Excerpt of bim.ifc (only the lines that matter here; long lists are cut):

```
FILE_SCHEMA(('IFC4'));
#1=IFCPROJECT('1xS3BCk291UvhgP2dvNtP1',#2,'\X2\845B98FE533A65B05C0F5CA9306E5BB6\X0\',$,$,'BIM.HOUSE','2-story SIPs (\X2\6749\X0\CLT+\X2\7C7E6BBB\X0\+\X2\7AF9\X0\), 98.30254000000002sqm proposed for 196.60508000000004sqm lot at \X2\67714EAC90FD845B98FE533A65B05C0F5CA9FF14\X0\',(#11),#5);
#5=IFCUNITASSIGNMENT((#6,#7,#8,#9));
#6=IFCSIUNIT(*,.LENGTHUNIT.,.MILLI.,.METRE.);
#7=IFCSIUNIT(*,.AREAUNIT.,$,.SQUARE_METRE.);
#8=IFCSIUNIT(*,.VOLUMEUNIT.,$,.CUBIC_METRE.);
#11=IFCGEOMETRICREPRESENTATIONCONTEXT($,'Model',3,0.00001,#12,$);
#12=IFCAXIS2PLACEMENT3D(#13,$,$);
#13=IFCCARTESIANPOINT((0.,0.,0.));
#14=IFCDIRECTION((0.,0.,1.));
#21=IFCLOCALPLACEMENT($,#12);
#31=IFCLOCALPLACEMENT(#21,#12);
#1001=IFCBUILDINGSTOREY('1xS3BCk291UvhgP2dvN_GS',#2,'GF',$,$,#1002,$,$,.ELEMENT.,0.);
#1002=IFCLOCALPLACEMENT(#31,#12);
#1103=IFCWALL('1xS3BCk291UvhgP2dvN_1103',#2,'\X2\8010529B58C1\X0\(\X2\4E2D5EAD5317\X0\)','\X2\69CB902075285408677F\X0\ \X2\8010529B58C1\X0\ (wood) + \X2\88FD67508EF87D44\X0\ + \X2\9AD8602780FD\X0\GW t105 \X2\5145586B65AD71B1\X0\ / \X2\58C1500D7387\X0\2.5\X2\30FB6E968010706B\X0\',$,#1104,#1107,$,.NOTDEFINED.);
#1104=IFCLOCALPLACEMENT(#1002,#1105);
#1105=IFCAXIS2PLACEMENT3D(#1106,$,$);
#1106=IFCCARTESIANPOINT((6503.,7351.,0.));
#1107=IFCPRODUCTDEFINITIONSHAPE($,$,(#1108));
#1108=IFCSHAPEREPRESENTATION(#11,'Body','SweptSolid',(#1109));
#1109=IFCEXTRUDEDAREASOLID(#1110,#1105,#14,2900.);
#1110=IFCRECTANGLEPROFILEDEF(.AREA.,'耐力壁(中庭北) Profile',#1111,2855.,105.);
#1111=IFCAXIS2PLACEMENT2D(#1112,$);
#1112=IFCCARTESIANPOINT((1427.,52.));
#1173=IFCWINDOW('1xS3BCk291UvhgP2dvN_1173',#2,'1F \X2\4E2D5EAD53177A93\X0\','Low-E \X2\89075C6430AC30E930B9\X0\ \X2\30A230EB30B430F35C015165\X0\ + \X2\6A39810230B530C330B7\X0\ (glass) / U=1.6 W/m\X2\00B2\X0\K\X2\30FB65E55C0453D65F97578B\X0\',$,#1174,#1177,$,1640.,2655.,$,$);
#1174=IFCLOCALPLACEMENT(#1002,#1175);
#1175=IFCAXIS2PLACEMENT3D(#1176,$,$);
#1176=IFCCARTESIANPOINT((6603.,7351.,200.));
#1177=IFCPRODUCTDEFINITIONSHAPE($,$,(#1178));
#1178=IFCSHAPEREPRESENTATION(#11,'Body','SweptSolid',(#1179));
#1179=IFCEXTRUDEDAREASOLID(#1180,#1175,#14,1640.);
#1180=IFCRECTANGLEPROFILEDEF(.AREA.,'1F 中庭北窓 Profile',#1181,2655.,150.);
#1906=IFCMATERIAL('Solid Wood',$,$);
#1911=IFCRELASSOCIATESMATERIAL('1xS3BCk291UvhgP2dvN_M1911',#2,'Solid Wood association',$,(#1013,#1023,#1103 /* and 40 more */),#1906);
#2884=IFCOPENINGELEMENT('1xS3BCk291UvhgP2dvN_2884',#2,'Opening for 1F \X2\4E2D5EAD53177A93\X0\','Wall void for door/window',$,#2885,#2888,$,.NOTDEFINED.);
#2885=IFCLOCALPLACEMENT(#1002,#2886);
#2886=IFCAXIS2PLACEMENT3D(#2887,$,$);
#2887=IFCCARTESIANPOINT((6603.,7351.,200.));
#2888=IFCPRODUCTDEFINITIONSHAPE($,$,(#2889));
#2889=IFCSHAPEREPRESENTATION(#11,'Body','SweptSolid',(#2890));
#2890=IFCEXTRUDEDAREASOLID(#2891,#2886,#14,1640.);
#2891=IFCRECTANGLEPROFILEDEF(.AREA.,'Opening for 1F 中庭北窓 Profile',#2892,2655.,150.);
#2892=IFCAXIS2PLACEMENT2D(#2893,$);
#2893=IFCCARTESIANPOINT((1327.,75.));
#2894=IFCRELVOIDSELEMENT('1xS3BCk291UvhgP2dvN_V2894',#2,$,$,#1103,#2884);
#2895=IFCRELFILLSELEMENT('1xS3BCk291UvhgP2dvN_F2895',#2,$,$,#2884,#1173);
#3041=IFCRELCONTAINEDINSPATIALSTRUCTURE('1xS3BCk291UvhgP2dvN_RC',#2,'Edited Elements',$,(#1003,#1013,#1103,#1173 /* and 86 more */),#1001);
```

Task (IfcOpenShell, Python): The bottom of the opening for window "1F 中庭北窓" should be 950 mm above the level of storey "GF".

```python
import numpy as np
import ifcopenshell
import ifcopenshell.api.geometry
import ifcopenshell.geom
import ifcopenshell.util.element
import ifcopenshell.util.placement
import ifcopenshell.util.shape
import ifcopenshell.util.unit

model = ifcopenshell.open("bim.ifc")
unit_scale = ifcopenshell.util.unit.calculate_unit_scale(model)

window = model.by_guid("1xS3BCk291UvhgP2dvN_1173")
opening = window.FillsVoids[0].RelatingOpeningElement
storey = ifcopenshell.util.element.get_container(window, ifc_class="IfcBuildingStorey")
level = ifcopenshell.util.placement.get_local_placement(storey.ObjectPlacement)[2, 3]

# The opening's origin need not be at the sill, so measure its lowest point.
shape = ifcopenshell.geom.create_shape(ifcopenshell.geom.settings(), opening)
bottom = ifcopenshell.util.shape.get_shape_bottom_elevation(shape, shape.geometry) / unit_scale
dz = level + 0.95 / unit_scale - bottom

shift = np.array([0.0, 0.0, dz])
# The window is not placed relative to its opening, so move both.
for product in (opening, window):
    matrix = ifcopenshell.util.placement.get_local_placement(product.ObjectPlacement)
    matrix[:3, 3] += shift
    ifcopenshell.api.geometry.edit_object_placement(model, product=product, matrix=matrix, is_si=False)

print(f"moved by {dz * unit_scale:+.3f} m")

model.write("bim_rev.ifc")
```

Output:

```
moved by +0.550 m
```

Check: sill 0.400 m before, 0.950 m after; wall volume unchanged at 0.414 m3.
